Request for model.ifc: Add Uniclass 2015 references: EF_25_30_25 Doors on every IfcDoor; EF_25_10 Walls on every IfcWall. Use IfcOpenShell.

First a look at what the model holds.

```python
import ifcopenshell

model = ifcopenshell.open("model.ifc")
print(model.schema)
print("classifications:", [c.Name for c in model.by_type("IfcClassification")])
for ifc_class in ("IfcDoor", "IfcRoof", "IfcStair", "IfcWall", "IfcWindow"):
    print(ifc_class, len(model.by_type(ifc_class)))
```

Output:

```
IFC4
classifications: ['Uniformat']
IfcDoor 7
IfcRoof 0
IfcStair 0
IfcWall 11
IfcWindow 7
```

```python
import ifcopenshell
import ifcopenshell.api.classification

model = ifcopenshell.open("model.ifc")

system = ifcopenshell.api.classification.add_classification(model, classification="Uniclass 2015")

codes = {
    "IfcDoor": ("EF_25_30_25", "Doors"),
    "IfcWall": ("EF_25_10", "Walls"),
}
for ifc_class, (code, name) in codes.items():
    products = model.by_type(ifc_class)
    ifcopenshell.api.classification.add_reference(
        model, products=products, classification=system, identification=code, name=name
    )
    print(code, len(products))

model.write("model_rev.ifc")
```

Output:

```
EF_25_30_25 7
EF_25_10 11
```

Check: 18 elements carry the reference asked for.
